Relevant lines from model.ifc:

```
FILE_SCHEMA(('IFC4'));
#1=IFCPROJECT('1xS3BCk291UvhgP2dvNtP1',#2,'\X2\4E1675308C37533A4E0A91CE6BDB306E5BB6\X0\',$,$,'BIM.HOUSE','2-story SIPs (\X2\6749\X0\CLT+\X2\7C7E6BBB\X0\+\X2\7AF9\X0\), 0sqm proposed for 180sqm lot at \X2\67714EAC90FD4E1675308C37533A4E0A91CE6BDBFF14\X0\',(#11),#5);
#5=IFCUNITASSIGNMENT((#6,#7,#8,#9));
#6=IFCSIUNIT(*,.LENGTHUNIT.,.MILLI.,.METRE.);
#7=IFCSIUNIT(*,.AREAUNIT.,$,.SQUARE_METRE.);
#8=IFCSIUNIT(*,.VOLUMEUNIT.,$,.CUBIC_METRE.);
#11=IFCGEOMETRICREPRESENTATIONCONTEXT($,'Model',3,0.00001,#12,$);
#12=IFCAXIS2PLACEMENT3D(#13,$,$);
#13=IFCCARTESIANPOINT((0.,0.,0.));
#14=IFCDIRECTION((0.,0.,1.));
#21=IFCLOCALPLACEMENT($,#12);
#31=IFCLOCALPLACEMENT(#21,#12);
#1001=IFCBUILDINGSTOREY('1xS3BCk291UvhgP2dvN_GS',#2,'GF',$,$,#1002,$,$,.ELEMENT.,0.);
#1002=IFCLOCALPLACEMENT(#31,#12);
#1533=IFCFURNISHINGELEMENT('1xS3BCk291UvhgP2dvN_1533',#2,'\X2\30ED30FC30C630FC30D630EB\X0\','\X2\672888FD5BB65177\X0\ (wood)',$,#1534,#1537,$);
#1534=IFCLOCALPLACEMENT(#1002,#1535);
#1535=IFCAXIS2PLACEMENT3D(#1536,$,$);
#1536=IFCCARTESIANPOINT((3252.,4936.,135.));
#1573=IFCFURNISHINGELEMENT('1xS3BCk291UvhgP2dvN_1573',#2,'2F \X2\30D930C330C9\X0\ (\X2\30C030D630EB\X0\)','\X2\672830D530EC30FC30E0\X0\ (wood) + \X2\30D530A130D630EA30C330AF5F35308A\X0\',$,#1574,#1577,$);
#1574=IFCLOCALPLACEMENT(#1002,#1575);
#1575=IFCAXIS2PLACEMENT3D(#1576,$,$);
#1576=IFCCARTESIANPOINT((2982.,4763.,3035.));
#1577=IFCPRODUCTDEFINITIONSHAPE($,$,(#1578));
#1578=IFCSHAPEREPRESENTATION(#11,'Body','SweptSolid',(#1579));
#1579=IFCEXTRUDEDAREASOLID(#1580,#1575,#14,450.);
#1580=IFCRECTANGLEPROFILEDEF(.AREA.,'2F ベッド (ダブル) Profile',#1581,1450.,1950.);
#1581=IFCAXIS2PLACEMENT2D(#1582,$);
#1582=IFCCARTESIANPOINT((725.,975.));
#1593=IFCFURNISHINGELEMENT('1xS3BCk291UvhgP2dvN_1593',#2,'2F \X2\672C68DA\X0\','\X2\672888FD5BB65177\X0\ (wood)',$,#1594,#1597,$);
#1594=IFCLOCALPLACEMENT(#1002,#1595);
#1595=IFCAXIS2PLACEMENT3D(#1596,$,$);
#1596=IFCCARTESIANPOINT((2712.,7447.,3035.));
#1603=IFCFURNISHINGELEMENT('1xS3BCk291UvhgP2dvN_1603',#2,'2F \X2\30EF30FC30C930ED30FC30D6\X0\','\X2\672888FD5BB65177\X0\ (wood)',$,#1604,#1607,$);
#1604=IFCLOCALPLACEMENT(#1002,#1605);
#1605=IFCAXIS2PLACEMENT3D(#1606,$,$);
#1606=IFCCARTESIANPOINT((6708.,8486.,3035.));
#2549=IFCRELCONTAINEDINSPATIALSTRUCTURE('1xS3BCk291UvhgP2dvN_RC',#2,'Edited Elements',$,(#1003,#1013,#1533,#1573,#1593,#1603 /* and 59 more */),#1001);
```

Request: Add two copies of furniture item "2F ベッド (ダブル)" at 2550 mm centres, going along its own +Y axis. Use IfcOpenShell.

```python
import ifcopenshell
import ifcopenshell.api.geometry
import ifcopenshell.api.root
import ifcopenshell.util.element
import ifcopenshell.util.placement
import ifcopenshell.util.unit

model = ifcopenshell.open("model.ifc")
unit_scale = ifcopenshell.util.unit.calculate_unit_scale(model)


def reuse_history(source, copy):
    """copy_class also copies each property set's owner history, people and application; keep the originals."""
    for rel in copy.IsDefinedBy:
        if rel.is_a("IfcRelDefinesByProperties") and (history := rel.RelatingPropertyDefinition.OwnerHistory):
            rel.RelatingPropertyDefinition.OwnerHistory = source.OwnerHistory
            ifcopenshell.util.element.remove_deep2(model, history)


source = model.by_guid("1xS3BCk291UvhgP2dvN_1573")
base = ifcopenshell.util.placement.get_local_placement(source.ObjectPlacement)
step = base[:3, 1] * 2.55 / unit_scale

for i in range(1, 3):
    copy = ifcopenshell.api.root.copy_class(model, product=source)
    copy.Representation = ifcopenshell.util.element.copy_deep(
        model, source.Representation, exclude=["IfcGeometricRepresentationContext", "IfcRepresentationMap"]
    )
    reuse_history(source, copy)
    matrix = base.copy()
    matrix[:3, 3] += i * step
    print("added at", matrix[:3, 3].round(3) + 0.0)
    ifcopenshell.api.geometry.edit_object_placement(model, product=copy, matrix=matrix, is_si=False)

model.write("model-out.ifc")
```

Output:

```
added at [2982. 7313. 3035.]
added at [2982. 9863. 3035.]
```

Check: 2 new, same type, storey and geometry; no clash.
